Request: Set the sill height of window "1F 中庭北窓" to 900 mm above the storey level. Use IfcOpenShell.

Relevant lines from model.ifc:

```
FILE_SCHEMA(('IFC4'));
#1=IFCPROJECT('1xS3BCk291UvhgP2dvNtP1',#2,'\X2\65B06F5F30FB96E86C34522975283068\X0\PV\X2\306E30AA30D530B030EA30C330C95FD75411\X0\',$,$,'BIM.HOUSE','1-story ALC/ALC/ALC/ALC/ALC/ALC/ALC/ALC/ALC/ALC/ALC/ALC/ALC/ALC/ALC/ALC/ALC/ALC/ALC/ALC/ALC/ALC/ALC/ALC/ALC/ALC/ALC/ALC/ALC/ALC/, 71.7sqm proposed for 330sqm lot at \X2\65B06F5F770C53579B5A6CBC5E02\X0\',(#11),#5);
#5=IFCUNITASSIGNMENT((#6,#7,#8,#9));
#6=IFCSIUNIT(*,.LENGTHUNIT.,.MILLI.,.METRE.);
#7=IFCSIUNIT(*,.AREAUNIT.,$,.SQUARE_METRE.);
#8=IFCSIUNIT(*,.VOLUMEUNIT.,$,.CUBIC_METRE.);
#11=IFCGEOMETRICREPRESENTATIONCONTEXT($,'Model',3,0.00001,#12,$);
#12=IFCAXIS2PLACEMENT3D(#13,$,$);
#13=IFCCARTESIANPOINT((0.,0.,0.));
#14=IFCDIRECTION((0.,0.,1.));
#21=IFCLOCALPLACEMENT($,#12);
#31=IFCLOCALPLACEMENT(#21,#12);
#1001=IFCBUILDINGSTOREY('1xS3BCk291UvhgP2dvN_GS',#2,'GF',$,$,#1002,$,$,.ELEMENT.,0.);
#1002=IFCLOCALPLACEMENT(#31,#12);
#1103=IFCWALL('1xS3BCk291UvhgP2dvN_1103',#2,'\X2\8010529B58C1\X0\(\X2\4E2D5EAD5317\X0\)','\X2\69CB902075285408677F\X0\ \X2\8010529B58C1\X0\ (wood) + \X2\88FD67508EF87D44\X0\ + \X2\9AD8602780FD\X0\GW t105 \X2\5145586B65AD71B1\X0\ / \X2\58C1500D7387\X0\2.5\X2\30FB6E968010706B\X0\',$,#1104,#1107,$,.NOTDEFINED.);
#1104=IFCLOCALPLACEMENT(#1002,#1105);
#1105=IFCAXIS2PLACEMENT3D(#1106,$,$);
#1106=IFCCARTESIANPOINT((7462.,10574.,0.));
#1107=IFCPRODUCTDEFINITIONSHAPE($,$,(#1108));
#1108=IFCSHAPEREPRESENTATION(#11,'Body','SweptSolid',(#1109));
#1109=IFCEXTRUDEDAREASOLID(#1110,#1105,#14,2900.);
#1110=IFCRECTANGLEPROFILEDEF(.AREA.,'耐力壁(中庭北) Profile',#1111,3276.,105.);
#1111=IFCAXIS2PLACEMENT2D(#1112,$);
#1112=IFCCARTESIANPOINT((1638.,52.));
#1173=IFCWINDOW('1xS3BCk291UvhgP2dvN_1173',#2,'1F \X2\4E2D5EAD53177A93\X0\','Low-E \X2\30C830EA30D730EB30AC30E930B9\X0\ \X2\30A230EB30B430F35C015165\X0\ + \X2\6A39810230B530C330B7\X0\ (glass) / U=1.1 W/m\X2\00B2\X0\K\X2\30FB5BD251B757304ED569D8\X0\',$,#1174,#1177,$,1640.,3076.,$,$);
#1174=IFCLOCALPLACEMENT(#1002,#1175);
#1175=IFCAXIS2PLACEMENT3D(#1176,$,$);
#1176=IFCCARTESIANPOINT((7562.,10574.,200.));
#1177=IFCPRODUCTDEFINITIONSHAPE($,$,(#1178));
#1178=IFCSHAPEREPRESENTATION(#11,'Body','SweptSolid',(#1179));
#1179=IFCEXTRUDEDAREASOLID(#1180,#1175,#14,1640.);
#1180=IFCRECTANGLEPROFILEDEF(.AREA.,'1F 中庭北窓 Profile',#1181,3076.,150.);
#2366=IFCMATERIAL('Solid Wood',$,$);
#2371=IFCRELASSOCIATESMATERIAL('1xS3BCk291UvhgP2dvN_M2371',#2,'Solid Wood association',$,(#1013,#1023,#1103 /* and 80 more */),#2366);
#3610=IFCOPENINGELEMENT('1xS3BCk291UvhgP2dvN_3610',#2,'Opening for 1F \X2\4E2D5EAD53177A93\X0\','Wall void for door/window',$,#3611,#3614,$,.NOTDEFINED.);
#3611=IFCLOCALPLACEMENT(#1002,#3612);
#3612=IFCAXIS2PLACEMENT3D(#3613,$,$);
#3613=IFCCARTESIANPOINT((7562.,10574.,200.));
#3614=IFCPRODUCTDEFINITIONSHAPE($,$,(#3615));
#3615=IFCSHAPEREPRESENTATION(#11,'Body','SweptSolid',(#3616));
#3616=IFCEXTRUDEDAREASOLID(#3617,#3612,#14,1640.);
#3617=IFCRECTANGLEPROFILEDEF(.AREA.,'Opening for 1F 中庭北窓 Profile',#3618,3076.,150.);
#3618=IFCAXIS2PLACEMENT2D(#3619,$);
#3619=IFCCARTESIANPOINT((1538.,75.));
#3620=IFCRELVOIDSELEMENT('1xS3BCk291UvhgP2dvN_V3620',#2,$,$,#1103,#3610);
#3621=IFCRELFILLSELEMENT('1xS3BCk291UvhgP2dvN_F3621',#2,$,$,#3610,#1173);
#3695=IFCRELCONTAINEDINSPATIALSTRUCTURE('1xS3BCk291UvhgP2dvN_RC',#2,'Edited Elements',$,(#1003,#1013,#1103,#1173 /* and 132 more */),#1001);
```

```python
import numpy as np
import ifcopenshell
import ifcopenshell.api.geometry
import ifcopenshell.geom
import ifcopenshell.util.element
import ifcopenshell.util.placement
import ifcopenshell.util.shape
import ifcopenshell.util.unit

model = ifcopenshell.open("model.ifc")
unit_scale = ifcopenshell.util.unit.calculate_unit_scale(model)

window = model.by_id(1173)
opening = window.FillsVoids[0].RelatingOpeningElement
storey = ifcopenshell.util.element.get_container(window, ifc_class="IfcBuildingStorey")
level = ifcopenshell.util.placement.get_local_placement(storey.ObjectPlacement)[2, 3]

# The opening's origin need not be at the sill, so measure its lowest point.
shape = ifcopenshell.geom.create_shape(ifcopenshell.geom.settings(), opening)
bottom = ifcopenshell.util.shape.get_shape_bottom_elevation(shape, shape.geometry) / unit_scale
dz = level + 0.9 / unit_scale - bottom

shift = np.array([0.0, 0.0, dz])
# The window is not placed relative to its opening, so move both.
for product in (opening, window):
    matrix = ifcopenshell.util.placement.get_local_placement(product.ObjectPlacement)
    matrix[:3, 3] += shift
    ifcopenshell.api.geometry.edit_object_placement(model, product=product, matrix=matrix, is_si=False)

print(f"moved by {dz * unit_scale:+.3f} m")

model.write("model_rev.ifc")
```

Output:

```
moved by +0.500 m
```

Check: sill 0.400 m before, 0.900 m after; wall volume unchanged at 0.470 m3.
